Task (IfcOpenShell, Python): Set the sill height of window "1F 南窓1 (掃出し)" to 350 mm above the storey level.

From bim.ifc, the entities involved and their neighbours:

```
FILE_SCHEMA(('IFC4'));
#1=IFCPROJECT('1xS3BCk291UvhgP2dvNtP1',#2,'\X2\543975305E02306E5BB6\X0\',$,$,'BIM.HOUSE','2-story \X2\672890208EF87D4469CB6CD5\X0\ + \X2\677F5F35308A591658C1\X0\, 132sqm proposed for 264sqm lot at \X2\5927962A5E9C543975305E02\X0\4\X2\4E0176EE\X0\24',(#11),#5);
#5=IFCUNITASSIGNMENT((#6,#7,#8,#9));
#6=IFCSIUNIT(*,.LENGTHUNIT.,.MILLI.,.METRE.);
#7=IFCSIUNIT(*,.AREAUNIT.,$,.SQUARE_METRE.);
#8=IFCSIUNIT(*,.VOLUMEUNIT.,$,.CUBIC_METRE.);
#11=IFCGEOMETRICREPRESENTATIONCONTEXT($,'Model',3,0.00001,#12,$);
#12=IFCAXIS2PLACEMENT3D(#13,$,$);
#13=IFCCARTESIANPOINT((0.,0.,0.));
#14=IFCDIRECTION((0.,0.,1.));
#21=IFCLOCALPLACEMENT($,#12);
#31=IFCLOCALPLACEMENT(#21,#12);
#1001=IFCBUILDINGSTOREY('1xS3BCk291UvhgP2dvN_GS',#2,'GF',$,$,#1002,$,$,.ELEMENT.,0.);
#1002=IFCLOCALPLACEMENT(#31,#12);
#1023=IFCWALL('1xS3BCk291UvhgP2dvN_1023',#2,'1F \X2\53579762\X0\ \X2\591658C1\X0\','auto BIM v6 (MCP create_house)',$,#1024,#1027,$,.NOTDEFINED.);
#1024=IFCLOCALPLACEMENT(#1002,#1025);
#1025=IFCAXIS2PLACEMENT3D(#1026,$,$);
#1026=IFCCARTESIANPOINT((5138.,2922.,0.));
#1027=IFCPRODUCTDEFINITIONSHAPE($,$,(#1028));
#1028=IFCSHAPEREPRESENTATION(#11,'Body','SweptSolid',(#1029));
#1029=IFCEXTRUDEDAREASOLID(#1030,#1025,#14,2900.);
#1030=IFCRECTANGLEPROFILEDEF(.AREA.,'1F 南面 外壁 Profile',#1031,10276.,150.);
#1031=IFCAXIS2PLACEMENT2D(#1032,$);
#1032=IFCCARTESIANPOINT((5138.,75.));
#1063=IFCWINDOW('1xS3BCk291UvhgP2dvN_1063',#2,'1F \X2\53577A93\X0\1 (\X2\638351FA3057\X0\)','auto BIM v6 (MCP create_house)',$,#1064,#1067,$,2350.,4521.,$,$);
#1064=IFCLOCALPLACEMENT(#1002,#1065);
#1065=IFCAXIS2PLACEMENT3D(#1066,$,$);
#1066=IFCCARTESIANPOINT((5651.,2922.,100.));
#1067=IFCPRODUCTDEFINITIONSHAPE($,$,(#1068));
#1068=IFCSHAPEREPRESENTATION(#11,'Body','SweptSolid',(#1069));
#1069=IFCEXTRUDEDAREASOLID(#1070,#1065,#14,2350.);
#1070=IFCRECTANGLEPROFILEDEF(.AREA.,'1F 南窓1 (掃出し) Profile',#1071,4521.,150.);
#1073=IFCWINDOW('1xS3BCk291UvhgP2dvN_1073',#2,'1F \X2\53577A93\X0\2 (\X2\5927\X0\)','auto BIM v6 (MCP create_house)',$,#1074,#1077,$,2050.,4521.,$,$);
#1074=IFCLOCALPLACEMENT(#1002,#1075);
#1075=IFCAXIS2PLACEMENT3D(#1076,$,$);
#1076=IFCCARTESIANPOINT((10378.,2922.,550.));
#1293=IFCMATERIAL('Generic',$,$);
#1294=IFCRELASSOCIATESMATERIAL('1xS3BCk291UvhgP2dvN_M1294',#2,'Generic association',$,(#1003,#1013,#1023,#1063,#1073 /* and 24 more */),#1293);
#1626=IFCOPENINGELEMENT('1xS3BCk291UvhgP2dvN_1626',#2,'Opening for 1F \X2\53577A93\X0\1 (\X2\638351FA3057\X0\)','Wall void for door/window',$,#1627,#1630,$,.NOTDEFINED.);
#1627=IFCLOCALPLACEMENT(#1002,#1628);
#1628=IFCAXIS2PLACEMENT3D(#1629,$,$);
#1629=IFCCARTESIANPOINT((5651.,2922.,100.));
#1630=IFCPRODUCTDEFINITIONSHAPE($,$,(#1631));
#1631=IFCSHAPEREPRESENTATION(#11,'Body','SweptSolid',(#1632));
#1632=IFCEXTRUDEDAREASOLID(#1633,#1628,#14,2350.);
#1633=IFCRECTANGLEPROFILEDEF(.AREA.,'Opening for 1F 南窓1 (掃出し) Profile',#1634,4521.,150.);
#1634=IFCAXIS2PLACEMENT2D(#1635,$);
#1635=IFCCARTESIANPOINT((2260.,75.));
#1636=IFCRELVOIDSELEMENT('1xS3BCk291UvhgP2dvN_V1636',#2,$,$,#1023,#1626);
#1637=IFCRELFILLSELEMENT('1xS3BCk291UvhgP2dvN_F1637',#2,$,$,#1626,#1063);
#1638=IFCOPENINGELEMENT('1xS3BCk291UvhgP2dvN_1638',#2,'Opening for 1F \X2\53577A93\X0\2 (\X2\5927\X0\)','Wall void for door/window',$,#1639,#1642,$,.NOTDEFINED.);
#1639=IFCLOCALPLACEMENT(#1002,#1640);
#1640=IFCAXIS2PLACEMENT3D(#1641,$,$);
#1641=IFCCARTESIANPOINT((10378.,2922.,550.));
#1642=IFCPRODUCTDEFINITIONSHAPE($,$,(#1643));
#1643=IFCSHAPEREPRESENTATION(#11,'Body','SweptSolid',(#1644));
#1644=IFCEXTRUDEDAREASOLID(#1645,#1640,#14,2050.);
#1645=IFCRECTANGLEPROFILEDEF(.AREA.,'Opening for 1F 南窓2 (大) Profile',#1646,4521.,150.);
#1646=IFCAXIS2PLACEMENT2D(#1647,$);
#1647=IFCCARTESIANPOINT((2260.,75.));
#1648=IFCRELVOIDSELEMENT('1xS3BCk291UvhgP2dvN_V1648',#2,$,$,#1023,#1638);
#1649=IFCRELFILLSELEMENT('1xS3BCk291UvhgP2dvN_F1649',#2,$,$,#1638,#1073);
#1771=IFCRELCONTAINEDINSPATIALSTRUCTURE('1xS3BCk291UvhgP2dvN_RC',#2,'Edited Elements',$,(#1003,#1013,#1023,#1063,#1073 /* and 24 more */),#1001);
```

```python
import numpy as np
import ifcopenshell
import ifcopenshell.api.geometry
import ifcopenshell.geom
import ifcopenshell.util.element
import ifcopenshell.util.placement
import ifcopenshell.util.shape
import ifcopenshell.util.unit

model = ifcopenshell.open("bim.ifc")
unit_scale = ifcopenshell.util.unit.calculate_unit_scale(model)

window = model.by_guid("1xS3BCk291UvhgP2dvN_1063")
opening = window.FillsVoids[0].RelatingOpeningElement
storey = ifcopenshell.util.element.get_container(window, ifc_class="IfcBuildingStorey")
level = ifcopenshell.util.placement.get_local_placement(storey.ObjectPlacement)[2, 3]

# The opening's origin need not be at the sill, so measure its lowest point.
shape = ifcopenshell.geom.create_shape(ifcopenshell.geom.settings(), opening)
bottom = ifcopenshell.util.shape.get_shape_bottom_elevation(shape, shape.geometry) / unit_scale
dz = level + 350.0 - bottom

shift = np.array([0.0, 0.0, dz])
# The window is not placed relative to its opening, so move both.
for product in (opening, window):
    matrix = ifcopenshell.util.placement.get_local_placement(product.ObjectPlacement)
    matrix[:3, 3] += shift
    ifcopenshell.api.geometry.edit_object_placement(model, product=product, matrix=matrix, is_si=False)

print(f"moved by {dz * unit_scale:+.3f} m")

model.write("bim_updated.ifc")
```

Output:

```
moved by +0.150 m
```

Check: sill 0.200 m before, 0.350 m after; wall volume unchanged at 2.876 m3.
